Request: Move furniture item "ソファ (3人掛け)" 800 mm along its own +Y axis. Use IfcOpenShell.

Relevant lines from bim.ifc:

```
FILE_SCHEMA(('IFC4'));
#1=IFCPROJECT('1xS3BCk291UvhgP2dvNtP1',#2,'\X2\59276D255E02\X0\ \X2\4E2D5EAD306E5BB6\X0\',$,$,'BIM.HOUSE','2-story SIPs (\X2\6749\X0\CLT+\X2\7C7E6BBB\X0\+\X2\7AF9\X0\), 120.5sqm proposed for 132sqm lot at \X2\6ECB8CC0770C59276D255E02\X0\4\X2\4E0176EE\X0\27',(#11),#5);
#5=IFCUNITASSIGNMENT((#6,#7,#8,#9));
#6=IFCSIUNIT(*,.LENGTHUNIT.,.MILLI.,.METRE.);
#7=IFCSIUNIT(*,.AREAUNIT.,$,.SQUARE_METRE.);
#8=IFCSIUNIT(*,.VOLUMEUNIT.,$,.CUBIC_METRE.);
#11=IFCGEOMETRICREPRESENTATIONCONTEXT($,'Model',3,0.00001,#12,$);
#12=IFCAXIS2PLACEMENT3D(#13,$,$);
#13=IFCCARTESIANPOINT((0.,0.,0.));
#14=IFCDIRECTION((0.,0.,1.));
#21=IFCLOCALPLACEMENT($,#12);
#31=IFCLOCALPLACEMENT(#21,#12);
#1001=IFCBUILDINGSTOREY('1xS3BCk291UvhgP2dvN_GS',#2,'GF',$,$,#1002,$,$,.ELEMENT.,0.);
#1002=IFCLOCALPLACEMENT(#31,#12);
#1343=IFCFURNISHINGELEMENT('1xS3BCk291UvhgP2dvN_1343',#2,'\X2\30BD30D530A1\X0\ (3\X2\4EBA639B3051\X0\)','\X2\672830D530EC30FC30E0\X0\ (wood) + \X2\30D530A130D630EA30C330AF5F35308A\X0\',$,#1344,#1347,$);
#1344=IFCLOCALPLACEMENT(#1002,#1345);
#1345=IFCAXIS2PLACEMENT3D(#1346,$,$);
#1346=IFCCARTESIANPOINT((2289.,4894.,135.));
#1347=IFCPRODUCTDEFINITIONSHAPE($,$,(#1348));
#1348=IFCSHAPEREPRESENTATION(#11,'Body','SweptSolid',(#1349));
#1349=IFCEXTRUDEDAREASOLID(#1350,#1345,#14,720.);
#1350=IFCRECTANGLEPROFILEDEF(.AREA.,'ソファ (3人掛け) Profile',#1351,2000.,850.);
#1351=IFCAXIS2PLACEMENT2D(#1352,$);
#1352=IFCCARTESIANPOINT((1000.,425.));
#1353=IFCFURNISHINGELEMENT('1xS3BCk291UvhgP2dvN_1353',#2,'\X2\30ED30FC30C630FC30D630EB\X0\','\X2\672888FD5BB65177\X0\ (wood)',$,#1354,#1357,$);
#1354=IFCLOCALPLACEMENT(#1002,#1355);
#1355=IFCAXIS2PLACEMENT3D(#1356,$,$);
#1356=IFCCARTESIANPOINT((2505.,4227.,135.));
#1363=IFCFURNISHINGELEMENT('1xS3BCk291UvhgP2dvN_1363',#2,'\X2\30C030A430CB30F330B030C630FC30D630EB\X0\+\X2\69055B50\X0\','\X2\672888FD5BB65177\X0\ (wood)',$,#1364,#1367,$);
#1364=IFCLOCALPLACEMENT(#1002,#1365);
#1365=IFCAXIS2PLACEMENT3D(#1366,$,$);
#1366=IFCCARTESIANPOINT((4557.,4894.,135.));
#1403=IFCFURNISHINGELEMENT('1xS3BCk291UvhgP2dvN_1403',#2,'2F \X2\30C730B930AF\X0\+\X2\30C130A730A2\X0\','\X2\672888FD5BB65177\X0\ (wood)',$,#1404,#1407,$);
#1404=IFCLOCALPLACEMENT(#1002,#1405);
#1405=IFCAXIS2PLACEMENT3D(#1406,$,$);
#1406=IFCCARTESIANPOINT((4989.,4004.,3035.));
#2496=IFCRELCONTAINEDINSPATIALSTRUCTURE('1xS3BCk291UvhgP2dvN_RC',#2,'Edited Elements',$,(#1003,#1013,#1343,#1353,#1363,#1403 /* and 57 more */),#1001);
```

```python
import ifcopenshell
import ifcopenshell.api.geometry
import ifcopenshell.util.placement
import ifcopenshell.util.unit

model = ifcopenshell.open("bim.ifc")
unit_scale = ifcopenshell.util.unit.calculate_unit_scale(model)

item = model.by_id(1343)
matrix = ifcopenshell.util.placement.get_local_placement(item.ObjectPlacement)
matrix[:3, 3] += matrix[:3, 1] * 0.8 / unit_scale
ifcopenshell.api.geometry.edit_object_placement(model, product=item, matrix=matrix, is_si=False)

print(ifcopenshell.util.placement.get_local_placement(item.ObjectPlacement).round(3) + 0.0)

model.write("bim_v2.ifc")
```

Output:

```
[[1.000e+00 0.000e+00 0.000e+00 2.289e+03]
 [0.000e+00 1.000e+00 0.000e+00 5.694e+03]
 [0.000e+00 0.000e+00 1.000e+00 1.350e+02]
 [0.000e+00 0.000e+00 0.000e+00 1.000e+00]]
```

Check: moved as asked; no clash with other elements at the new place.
